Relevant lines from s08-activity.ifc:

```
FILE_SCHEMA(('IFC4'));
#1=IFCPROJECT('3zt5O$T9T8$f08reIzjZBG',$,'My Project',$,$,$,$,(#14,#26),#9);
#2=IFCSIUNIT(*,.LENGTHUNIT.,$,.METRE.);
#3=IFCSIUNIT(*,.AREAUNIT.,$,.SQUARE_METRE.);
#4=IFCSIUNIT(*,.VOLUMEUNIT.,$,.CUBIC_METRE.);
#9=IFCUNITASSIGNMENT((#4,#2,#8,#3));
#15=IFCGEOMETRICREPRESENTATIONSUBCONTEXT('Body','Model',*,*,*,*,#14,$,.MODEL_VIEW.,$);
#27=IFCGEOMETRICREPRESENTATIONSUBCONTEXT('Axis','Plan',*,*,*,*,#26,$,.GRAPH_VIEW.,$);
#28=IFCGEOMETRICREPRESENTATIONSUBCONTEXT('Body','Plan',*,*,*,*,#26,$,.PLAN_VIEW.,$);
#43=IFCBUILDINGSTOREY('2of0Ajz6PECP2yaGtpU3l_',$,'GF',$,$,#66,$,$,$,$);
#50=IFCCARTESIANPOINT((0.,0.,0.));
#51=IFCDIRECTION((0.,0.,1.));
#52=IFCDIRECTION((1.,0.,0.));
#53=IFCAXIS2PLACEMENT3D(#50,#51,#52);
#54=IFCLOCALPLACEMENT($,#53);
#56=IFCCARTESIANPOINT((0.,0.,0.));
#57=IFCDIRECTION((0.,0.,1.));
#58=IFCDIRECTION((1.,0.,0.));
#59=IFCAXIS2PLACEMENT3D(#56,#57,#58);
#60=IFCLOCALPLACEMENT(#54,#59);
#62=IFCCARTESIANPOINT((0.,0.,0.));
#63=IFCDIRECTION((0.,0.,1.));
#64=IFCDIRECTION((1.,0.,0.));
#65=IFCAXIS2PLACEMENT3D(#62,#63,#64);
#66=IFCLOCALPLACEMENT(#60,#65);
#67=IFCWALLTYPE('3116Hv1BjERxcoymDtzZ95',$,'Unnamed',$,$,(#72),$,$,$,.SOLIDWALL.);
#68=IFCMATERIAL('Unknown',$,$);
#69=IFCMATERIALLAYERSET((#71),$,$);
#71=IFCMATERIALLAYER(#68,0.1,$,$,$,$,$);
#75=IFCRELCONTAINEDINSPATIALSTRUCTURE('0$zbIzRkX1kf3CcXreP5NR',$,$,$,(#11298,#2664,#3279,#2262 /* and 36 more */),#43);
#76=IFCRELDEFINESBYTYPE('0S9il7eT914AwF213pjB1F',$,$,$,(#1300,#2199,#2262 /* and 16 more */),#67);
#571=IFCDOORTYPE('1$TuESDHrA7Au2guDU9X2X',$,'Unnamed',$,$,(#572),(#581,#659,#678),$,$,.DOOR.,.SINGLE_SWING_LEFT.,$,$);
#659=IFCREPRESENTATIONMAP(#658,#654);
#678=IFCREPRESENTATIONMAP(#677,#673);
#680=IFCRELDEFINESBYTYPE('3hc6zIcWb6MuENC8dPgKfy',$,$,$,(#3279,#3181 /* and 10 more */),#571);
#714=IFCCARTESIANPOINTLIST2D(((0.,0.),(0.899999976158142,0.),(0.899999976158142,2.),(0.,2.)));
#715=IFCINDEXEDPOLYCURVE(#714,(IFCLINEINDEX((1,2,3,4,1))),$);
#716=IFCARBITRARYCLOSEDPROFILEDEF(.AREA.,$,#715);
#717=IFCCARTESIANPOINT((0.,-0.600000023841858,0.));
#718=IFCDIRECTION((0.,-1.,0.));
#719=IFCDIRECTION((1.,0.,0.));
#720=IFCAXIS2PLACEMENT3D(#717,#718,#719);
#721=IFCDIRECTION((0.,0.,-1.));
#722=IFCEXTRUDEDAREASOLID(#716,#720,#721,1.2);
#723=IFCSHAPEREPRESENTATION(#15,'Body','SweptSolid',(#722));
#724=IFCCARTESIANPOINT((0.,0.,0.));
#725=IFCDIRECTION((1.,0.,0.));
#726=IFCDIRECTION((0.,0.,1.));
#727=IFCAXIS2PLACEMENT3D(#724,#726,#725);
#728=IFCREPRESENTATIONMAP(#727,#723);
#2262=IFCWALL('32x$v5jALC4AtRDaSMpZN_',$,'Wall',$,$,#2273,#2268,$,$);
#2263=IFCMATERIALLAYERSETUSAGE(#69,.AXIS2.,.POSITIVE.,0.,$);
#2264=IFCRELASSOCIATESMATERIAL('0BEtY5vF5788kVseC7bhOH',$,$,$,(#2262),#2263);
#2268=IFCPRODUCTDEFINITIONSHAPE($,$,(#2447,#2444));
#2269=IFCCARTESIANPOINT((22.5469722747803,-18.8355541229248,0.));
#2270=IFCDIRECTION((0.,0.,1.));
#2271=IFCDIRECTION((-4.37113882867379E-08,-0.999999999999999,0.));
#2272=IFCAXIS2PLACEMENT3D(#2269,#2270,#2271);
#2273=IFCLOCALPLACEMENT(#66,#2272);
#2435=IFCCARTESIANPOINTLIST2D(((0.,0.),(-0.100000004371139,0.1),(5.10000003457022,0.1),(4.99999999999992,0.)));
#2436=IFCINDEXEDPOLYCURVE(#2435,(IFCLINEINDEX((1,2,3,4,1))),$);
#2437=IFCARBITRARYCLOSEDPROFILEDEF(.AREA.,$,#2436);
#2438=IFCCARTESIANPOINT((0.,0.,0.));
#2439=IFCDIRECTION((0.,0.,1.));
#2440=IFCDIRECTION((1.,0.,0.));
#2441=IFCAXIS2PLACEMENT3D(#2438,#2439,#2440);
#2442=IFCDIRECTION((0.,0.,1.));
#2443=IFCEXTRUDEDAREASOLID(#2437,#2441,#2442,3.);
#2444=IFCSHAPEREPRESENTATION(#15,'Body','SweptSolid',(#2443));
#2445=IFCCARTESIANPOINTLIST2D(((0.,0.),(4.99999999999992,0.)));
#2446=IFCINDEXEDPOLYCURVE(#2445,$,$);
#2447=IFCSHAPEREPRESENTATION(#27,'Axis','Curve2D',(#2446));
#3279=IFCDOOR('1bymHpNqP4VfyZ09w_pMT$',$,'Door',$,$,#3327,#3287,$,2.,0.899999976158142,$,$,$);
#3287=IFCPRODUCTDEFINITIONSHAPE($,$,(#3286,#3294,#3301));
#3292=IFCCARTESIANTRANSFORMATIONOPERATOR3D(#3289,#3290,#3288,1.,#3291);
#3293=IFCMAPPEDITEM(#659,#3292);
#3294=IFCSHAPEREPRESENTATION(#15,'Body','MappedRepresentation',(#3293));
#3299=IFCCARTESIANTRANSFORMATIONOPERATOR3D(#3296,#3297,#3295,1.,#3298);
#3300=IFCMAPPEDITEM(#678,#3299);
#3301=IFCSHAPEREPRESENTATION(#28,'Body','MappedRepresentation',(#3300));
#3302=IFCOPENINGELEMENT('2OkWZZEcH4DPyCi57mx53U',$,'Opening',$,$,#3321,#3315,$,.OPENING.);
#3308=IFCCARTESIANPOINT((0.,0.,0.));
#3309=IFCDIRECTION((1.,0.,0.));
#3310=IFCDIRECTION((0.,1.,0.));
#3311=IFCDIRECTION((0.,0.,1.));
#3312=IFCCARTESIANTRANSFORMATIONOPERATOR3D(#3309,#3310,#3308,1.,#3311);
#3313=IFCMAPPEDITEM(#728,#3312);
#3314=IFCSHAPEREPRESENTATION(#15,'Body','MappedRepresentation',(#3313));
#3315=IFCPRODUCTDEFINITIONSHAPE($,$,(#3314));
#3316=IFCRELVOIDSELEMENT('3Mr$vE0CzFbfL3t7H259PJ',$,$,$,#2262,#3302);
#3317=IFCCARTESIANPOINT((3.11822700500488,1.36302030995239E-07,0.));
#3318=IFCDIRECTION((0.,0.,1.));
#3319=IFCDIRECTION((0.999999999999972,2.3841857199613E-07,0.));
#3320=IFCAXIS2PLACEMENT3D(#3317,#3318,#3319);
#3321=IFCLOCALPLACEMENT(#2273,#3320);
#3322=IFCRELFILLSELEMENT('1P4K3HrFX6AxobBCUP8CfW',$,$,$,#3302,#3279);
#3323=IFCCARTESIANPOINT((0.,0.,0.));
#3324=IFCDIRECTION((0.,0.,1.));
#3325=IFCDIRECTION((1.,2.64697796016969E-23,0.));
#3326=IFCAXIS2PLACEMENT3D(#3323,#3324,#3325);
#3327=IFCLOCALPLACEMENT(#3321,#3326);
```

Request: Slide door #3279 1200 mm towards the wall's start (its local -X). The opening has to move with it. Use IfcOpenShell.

```python
import ifcopenshell
import ifcopenshell.api.geometry
import ifcopenshell.util.placement
import ifcopenshell.util.unit

model = ifcopenshell.open("s08-activity.ifc")
unit_scale = ifcopenshell.util.unit.calculate_unit_scale(model)

door = model.by_guid("1bymHpNqP4VfyZ09w_pMT$")
opening = door.FillsVoids[0].RelatingOpeningElement
wall = opening.VoidsElements[0].RelatingBuildingElement

wall_matrix = ifcopenshell.util.placement.get_local_placement(wall.ObjectPlacement)
shift = wall_matrix[:3, 0] * -1.2 / unit_scale
before = ifcopenshell.util.placement.get_local_placement(door.ObjectPlacement)[:3, 3].copy()

# The door is placed relative to its opening, so it follows when the opening moves.
matrix = ifcopenshell.util.placement.get_local_placement(opening.ObjectPlacement)
matrix[:3, 3] += shift
ifcopenshell.api.geometry.edit_object_placement(
    model, product=opening, matrix=matrix, is_si=False, should_transform_children=True
)

after = ifcopenshell.util.placement.get_local_placement(door.ObjectPlacement)[:3, 3]
print("door moved by", (after - before).round(3) + 0.0)

model.write("s08-activity_rev.ifc")
```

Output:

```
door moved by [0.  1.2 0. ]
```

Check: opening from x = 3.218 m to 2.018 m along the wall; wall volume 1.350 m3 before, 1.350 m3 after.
